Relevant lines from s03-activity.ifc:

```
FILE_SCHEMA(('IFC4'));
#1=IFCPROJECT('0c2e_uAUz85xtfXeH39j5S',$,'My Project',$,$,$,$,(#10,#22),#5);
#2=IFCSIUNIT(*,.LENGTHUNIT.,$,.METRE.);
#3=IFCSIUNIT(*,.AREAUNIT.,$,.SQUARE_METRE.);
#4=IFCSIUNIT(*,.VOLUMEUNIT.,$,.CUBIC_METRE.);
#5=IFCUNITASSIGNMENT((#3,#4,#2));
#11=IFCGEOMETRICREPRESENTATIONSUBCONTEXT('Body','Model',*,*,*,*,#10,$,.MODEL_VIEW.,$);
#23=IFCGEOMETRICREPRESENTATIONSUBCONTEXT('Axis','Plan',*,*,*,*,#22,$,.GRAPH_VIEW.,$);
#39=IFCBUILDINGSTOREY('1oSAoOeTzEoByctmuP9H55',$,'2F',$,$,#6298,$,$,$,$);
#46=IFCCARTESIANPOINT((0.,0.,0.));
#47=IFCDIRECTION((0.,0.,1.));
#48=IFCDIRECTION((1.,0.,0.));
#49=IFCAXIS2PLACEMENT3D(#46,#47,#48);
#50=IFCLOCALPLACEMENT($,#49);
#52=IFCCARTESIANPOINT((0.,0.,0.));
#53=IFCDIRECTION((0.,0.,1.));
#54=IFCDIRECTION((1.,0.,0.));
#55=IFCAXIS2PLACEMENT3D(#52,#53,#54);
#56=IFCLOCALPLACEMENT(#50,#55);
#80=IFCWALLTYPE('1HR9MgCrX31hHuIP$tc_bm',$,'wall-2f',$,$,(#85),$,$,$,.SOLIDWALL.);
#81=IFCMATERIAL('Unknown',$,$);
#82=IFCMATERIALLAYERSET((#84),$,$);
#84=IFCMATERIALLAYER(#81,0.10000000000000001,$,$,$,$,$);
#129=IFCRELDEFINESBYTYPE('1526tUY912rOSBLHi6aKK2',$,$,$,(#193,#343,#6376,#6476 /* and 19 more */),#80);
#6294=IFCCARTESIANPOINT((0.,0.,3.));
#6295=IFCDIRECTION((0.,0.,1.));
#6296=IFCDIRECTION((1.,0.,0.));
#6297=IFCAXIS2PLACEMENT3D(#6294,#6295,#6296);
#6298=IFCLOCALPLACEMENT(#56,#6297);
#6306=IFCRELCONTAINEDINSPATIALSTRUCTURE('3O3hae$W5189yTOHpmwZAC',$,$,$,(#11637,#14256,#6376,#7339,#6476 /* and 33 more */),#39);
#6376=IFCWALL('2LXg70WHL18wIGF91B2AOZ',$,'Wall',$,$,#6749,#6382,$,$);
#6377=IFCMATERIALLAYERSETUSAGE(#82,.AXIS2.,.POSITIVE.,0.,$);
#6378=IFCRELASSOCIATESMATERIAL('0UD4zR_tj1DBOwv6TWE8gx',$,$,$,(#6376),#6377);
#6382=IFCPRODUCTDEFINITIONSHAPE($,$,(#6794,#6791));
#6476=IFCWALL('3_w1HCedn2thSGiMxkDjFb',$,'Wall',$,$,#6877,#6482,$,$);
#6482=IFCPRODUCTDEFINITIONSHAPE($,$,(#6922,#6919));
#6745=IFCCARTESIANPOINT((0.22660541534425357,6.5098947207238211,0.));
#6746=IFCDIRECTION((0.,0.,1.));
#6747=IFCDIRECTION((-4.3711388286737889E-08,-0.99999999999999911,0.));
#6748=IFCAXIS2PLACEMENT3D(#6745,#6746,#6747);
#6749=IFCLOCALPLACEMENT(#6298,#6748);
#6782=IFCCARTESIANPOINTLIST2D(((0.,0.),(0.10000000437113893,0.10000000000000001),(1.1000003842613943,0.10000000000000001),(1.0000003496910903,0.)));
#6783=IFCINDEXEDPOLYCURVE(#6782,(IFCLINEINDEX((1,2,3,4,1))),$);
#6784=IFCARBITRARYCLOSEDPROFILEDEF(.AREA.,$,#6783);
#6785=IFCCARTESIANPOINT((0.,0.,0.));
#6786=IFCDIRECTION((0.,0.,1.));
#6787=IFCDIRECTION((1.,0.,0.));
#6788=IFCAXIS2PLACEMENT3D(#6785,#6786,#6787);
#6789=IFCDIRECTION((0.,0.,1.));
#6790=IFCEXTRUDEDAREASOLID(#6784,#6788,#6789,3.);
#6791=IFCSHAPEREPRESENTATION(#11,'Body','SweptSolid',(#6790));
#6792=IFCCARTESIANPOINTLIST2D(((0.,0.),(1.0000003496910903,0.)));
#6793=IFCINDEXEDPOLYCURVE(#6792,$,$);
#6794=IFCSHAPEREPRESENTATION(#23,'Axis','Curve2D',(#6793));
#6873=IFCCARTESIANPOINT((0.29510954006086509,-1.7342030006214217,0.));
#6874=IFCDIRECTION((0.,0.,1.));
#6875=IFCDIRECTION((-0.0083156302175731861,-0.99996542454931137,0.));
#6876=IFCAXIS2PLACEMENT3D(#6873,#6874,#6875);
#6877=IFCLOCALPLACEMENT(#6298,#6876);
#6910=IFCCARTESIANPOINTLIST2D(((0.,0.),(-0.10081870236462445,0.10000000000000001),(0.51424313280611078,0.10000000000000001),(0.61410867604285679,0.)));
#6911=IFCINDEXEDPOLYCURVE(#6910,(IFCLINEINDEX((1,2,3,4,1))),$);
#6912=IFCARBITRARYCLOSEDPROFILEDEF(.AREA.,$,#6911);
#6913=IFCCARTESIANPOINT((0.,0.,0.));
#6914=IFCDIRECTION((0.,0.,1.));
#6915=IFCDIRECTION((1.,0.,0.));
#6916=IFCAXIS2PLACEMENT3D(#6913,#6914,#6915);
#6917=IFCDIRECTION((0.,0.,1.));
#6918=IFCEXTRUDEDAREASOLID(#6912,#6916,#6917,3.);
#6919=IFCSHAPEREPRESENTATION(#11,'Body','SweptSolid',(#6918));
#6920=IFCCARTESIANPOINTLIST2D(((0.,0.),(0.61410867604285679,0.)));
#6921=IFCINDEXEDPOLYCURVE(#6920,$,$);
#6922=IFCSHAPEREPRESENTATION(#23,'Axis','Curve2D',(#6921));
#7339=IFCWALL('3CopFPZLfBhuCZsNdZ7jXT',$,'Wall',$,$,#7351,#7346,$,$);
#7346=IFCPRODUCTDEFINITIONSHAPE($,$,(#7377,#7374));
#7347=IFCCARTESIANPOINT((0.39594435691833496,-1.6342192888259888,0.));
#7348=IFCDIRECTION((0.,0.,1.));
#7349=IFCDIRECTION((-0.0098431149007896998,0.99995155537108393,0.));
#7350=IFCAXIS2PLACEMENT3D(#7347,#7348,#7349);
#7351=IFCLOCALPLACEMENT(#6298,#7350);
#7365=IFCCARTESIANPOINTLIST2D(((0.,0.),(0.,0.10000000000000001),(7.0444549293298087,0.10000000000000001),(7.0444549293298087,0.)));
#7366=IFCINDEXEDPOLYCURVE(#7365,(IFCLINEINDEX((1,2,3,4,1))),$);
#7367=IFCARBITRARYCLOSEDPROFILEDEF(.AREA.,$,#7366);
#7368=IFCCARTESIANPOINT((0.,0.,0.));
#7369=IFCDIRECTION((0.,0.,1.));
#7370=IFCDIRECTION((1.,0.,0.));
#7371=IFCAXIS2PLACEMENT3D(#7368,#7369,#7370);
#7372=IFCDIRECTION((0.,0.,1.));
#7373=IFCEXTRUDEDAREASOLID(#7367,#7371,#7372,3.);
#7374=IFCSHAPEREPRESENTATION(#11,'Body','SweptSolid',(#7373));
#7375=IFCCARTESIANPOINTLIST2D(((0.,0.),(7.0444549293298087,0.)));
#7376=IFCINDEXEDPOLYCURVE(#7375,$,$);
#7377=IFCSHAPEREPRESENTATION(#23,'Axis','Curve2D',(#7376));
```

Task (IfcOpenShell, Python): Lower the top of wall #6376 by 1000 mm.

```python
import ifcopenshell
import ifcopenshell.geom
import ifcopenshell.util.representation
import ifcopenshell.util.shape

model = ifcopenshell.open("s03-activity.ifc")
settings = ifcopenshell.geom.settings()


def volume(element):
    """Net volume in cubic metres, openings subtracted."""
    shape = ifcopenshell.geom.create_shape(settings, element)
    return ifcopenshell.util.shape.get_volume(shape.geometry)


wall = model.by_id(6376)
before = volume(wall)

body = ifcopenshell.util.representation.get_representation(wall, "Model", "Body")
solid = body.Items[0]
old_height = solid.Depth
solid.Depth -= 1.0
after = volume(wall)

print(f"height {old_height:g} -> {solid.Depth:g}, volume {before:.3f} -> {after:.3f} m3")

model.write("s03-activity_updated.ifc")
```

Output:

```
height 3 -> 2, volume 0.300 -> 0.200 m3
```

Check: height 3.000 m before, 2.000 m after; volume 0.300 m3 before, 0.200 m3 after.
